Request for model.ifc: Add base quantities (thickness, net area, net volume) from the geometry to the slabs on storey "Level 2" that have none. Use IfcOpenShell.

First a look at what the model holds.

```python
import ifcopenshell
import ifcopenshell.util.element
import ifcopenshell.util.unit

model = ifcopenshell.open("model.ifc")
print(model.schema)
for unit_type in ("LENGTHUNIT", "AREAUNIT", "VOLUMEUNIT"):
    print(unit_type, ifcopenshell.util.unit.calculate_unit_scale(model, unit_type))
storey = next(s for s in model.by_type("IfcBuildingStorey") if s.Name == "Level 2")
slabs = [e for e in ifcopenshell.util.element.get_decomposition(storey) if e.is_a("IfcSlab")]
for e in sorted(slabs, key=lambda e: e.id()):
    print(e.id(), e.is_a(), e.Name, list(ifcopenshell.util.element.get_psets(e, qtos_only=True)), sep=" | ")
```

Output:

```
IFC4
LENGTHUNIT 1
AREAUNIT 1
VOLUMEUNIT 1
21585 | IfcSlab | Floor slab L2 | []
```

```python
import ifcopenshell
import ifcopenshell.api.pset
import ifcopenshell.geom
import ifcopenshell.util.element
import ifcopenshell.util.shape
import ifcopenshell.util.unit

model = ifcopenshell.open("model.ifc")
unit_scale = ifcopenshell.util.unit.calculate_unit_scale(model)
area_scale = ifcopenshell.util.unit.calculate_unit_scale(model, "AREAUNIT")
volume_scale = ifcopenshell.util.unit.calculate_unit_scale(model, "VOLUMEUNIT")
settings = ifcopenshell.geom.settings()

storey = next(s for s in model.by_type("IfcBuildingStorey") if s.Name == "Level 2")
slabs = [e for e in ifcopenshell.util.element.get_decomposition(storey) if e.is_a("IfcSlab")]

for e in sorted(slabs, key=lambda e: e.id()):
    if ifcopenshell.util.element.get_psets(e, qtos_only=True, should_inherit=False):
        continue
    # Geometry comes back in metres, in the element's own axes.
    shape = ifcopenshell.geom.create_shape(settings, e)
    values = {
        "Width": ifcopenshell.util.shape.get_z(shape.geometry) / unit_scale,
        "NetArea": ifcopenshell.util.shape.get_footprint_area(shape.geometry) / area_scale,
        "NetVolume": ifcopenshell.util.shape.get_volume(shape.geometry) / volume_scale,
    }
    qto = ifcopenshell.api.pset.add_qto(model, product=e, name="Qto_SlabBaseQuantities")
    ifcopenshell.api.pset.edit_qto(model, qto=qto, properties=values)
    print(e.id(), {k: round(v, 3) for k, v in values.items()})

model.write("model_edited.ifc")
```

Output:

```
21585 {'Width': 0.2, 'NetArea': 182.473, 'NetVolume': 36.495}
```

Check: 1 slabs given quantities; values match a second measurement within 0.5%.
